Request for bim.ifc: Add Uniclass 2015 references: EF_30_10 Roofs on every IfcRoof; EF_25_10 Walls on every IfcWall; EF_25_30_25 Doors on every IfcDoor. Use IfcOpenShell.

First a look at what the model holds.

```python
import ifcopenshell

model = ifcopenshell.open("bim.ifc")
print(model.schema)
print("classifications:", [c.Name for c in model.by_type("IfcClassification")])
for ifc_class in ("IfcDoor", "IfcRoof", "IfcStair", "IfcWall", "IfcWindow"):
    print(ifc_class, len(model.by_type(ifc_class)))
```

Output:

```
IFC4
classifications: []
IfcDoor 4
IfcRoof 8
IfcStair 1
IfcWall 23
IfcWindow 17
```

```python
import ifcopenshell
import ifcopenshell.api.classification

model = ifcopenshell.open("bim.ifc")

system = ifcopenshell.api.classification.add_classification(model, classification="Uniclass 2015")

codes = {
    "IfcRoof": ("EF_30_10", "Roofs"),
    "IfcWall": ("EF_25_10", "Walls"),
    "IfcDoor": ("EF_25_30_25", "Doors"),
}
for ifc_class, (code, name) in codes.items():
    products = model.by_type(ifc_class)
    ifcopenshell.api.classification.add_reference(
        model, products=products, classification=system, identification=code, name=name
    )
    print(code, len(products))

model.write("bim_updated.ifc")
```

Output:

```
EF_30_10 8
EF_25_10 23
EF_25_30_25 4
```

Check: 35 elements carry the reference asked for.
